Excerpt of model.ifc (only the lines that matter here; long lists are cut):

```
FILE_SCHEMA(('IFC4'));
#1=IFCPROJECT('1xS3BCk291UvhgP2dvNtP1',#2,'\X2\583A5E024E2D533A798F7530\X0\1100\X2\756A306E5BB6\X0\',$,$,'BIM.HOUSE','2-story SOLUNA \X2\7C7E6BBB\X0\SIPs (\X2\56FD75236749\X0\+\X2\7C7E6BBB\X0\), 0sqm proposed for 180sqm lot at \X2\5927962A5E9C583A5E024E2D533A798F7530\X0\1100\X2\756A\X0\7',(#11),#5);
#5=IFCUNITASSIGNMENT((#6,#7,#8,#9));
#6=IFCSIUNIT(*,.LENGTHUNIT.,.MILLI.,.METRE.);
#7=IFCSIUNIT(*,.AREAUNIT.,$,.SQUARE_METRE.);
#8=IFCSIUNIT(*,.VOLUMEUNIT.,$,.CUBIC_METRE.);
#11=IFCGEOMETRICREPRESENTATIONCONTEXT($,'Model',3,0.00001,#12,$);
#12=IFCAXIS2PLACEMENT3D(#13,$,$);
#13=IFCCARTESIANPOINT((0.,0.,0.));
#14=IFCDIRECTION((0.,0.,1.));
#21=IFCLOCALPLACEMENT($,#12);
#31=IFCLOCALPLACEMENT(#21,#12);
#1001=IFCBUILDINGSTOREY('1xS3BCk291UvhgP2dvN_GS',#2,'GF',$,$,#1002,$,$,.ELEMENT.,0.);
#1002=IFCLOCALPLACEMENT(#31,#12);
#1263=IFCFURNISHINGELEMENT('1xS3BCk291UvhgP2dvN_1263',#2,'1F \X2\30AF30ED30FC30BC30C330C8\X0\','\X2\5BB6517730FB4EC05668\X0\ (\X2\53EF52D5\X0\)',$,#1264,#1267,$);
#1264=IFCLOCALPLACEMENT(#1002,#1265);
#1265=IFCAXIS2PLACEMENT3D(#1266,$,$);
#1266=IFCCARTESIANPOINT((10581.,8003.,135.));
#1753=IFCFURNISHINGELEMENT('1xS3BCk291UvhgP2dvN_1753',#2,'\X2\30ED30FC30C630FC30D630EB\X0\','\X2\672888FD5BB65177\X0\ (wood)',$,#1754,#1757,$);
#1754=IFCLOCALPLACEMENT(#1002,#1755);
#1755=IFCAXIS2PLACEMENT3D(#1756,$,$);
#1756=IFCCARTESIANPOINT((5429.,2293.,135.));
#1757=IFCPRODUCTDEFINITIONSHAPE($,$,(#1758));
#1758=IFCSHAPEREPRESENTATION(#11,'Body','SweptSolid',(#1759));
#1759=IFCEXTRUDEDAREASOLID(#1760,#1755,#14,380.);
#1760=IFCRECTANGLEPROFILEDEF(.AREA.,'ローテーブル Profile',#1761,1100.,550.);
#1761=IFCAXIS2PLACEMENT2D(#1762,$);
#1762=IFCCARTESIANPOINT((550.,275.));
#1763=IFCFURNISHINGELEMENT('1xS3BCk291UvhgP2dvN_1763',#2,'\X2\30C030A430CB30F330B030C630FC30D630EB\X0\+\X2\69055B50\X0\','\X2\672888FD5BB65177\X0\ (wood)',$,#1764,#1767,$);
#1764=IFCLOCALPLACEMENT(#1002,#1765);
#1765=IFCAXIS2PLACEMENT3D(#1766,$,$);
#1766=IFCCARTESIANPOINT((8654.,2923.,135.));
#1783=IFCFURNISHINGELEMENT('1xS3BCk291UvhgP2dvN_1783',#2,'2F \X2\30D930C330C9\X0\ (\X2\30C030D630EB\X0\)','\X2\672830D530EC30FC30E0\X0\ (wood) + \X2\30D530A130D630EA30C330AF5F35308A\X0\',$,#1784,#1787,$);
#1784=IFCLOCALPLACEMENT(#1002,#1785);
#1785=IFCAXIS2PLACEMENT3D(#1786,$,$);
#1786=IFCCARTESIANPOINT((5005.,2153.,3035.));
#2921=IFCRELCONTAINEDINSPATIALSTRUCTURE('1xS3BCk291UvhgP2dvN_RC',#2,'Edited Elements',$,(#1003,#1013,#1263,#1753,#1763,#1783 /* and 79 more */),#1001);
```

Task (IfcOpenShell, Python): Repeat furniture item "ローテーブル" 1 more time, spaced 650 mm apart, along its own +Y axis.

```python
import ifcopenshell
import ifcopenshell.api.geometry
import ifcopenshell.api.root
import ifcopenshell.util.element
import ifcopenshell.util.placement

model = ifcopenshell.open("model.ifc")


def reuse_history(source, copy):
    """copy_class also copies each property set's owner history, people and application; keep the originals."""
    for rel in copy.IsDefinedBy:
        if rel.is_a("IfcRelDefinesByProperties") and (history := rel.RelatingPropertyDefinition.OwnerHistory):
            rel.RelatingPropertyDefinition.OwnerHistory = source.OwnerHistory
            ifcopenshell.util.element.remove_deep2(model, history)


source = model.by_id(1753)
base = ifcopenshell.util.placement.get_local_placement(source.ObjectPlacement)
step = base[:3, 1] * 650.0

for i in range(1, 2):
    copy = ifcopenshell.api.root.copy_class(model, product=source)
    copy.Representation = ifcopenshell.util.element.copy_deep(
        model, source.Representation, exclude=["IfcGeometricRepresentationContext", "IfcRepresentationMap"]
    )
    reuse_history(source, copy)
    matrix = base.copy()
    matrix[:3, 3] += i * step
    print("added at", matrix[:3, 3].round(3) + 0.0)
    ifcopenshell.api.geometry.edit_object_placement(model, product=copy, matrix=matrix, is_si=False)

model.write("model_updated.ifc")
```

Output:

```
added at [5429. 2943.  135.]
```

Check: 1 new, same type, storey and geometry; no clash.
